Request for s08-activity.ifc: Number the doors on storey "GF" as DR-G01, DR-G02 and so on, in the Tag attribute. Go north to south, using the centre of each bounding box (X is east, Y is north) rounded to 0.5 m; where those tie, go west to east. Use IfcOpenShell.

First a look at what the model holds.

```python
import ifcopenshell
import ifcopenshell.util.element
import ifcopenshell.util.placement

model = ifcopenshell.open("s08-activity.ifc")
print(model.schema)
storey = next(s for s in model.by_type("IfcBuildingStorey") if s.Name == "GF")
doors = [e for e in ifcopenshell.util.element.get_decomposition(storey) if e.is_a("IfcDoor")]
for e in sorted(doors, key=lambda e: e.id()):
    origin = ifcopenshell.util.placement.get_local_placement(e.ObjectPlacement)[:3, 3]
    print(e.id(), e.Tag, e.Name, origin.round(2) + 0.0, sep=" | ")
```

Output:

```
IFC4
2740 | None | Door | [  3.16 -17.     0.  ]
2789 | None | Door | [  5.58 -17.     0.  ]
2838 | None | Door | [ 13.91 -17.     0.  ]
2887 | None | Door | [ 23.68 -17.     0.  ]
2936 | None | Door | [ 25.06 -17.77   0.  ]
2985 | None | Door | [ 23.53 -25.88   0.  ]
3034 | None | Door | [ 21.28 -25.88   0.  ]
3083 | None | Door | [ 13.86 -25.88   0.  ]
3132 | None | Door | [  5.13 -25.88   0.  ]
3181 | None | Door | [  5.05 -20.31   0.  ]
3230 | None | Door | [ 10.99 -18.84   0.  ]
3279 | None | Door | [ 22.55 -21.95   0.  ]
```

```python
import ifcopenshell
import ifcopenshell.geom
import ifcopenshell.util.element
import ifcopenshell.util.shape

model = ifcopenshell.open("s08-activity.ifc")
settings = ifcopenshell.geom.settings()
settings.set("use-world-coords", True)


def centre(element):
    shape = ifcopenshell.geom.create_shape(settings, element)
    return ifcopenshell.util.shape.get_bbox_centroid(shape.geometry)


storey = next(s for s in model.by_type("IfcBuildingStorey") if s.Name == "GF")
doors = [e for e in ifcopenshell.util.element.get_decomposition(storey) if e.is_a("IfcDoor")]

# Insertion points can sit at a corner or the storey origin, so sort by the geometry (in metres).
centres = {e: centre(e) for e in doors}
doors.sort(key=lambda e: (-round(centres[e][1] / 0.5), centres[e][0]))

for i, e in enumerate(doors, start=1):
    number = f"DR-G{i:02d}"
    e.Tag = number
    print(e.id(), number)

model.write("s08-activity-out.ifc")
```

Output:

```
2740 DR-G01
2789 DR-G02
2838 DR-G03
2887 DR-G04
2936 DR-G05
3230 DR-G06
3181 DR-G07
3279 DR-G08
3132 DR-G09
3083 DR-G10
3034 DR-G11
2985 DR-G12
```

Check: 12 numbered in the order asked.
